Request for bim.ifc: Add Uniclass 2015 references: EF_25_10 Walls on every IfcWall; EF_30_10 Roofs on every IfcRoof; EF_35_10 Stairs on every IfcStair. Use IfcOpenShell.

First a look at what the model holds.

```python
import ifcopenshell

model = ifcopenshell.open("bim.ifc")
print(model.schema)
print("classifications:", [c.Name for c in model.by_type("IfcClassification")])
for ifc_class in ("IfcDoor", "IfcRoof", "IfcStair", "IfcWall", "IfcWindow"):
    print(ifc_class, len(model.by_type(ifc_class)))
```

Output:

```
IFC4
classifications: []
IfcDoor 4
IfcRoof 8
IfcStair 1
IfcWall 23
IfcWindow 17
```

```python
import ifcopenshell
import ifcopenshell.api.classification

model = ifcopenshell.open("bim.ifc")

system = ifcopenshell.api.classification.add_classification(model, classification="Uniclass 2015")

codes = {
    "IfcWall": ("EF_25_10", "Walls"),
    "IfcRoof": ("EF_30_10", "Roofs"),
    "IfcStair": ("EF_35_10", "Stairs"),
}
for ifc_class, (code, name) in codes.items():
    products = model.by_type(ifc_class)
    ifcopenshell.api.classification.add_reference(
        model, products=products, classification=system, identification=code, name=name
    )
    print(code, len(products))

model.write("bim_v2.ifc")
```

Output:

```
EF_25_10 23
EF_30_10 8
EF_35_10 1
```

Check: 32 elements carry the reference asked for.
